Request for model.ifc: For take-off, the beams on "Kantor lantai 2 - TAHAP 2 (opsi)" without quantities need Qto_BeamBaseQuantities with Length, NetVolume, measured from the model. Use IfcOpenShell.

First a look at what the model holds.

```python
import ifcopenshell
import ifcopenshell.util.element
import ifcopenshell.util.unit

model = ifcopenshell.open("model.ifc")
print(model.schema)
for unit_type in ("LENGTHUNIT", "AREAUNIT", "VOLUMEUNIT"):
    print(unit_type, ifcopenshell.util.unit.calculate_unit_scale(model, unit_type))
storey = next(s for s in model.by_type("IfcBuildingStorey") if s.Name == "Kantor lantai 2 - TAHAP 2 (opsi)")
beams = [e for e in ifcopenshell.util.element.get_decomposition(storey) if e.is_a("IfcBeam")]
for e in sorted(beams, key=lambda e: e.id()):
    print(e.id(), e.is_a(), e.Name, list(ifcopenshell.util.element.get_psets(e, qtos_only=True)), sep=" | ")
```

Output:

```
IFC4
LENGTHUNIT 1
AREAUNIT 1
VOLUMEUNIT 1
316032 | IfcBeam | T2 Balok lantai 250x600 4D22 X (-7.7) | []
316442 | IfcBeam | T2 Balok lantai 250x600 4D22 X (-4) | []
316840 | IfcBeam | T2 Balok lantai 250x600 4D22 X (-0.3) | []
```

```python
import ifcopenshell
import ifcopenshell.api.pset
import ifcopenshell.geom
import ifcopenshell.util.element
import ifcopenshell.util.shape
import ifcopenshell.util.unit

model = ifcopenshell.open("model.ifc")
unit_scale = ifcopenshell.util.unit.calculate_unit_scale(model)
volume_scale = ifcopenshell.util.unit.calculate_unit_scale(model, "VOLUMEUNIT")
settings = ifcopenshell.geom.settings()

storey = next(s for s in model.by_type("IfcBuildingStorey") if s.Name == "Kantor lantai 2 - TAHAP 2 (opsi)")
beams = [e for e in ifcopenshell.util.element.get_decomposition(storey) if e.is_a("IfcBeam")]

for e in sorted(beams, key=lambda e: e.id()):
    if ifcopenshell.util.element.get_psets(e, qtos_only=True, should_inherit=False):
        continue
    # Geometry comes back in metres, in the element's own axes.
    shape = ifcopenshell.geom.create_shape(settings, e)
    values = {
        "Length": ifcopenshell.util.shape.get_max_xyz(shape.geometry) / unit_scale,
        "NetVolume": ifcopenshell.util.shape.get_volume(shape.geometry) / volume_scale,
    }
    qto = ifcopenshell.api.pset.add_qto(model, product=e, name="Qto_BeamBaseQuantities")
    ifcopenshell.api.pset.edit_qto(model, qto=qto, properties=values)
    print(e.id(), {k: round(v, 3) for k, v in values.items()})

model.write("model_rev.ifc")
```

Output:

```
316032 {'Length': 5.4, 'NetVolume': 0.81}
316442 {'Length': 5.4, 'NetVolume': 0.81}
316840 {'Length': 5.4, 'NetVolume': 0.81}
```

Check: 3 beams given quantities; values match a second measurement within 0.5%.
